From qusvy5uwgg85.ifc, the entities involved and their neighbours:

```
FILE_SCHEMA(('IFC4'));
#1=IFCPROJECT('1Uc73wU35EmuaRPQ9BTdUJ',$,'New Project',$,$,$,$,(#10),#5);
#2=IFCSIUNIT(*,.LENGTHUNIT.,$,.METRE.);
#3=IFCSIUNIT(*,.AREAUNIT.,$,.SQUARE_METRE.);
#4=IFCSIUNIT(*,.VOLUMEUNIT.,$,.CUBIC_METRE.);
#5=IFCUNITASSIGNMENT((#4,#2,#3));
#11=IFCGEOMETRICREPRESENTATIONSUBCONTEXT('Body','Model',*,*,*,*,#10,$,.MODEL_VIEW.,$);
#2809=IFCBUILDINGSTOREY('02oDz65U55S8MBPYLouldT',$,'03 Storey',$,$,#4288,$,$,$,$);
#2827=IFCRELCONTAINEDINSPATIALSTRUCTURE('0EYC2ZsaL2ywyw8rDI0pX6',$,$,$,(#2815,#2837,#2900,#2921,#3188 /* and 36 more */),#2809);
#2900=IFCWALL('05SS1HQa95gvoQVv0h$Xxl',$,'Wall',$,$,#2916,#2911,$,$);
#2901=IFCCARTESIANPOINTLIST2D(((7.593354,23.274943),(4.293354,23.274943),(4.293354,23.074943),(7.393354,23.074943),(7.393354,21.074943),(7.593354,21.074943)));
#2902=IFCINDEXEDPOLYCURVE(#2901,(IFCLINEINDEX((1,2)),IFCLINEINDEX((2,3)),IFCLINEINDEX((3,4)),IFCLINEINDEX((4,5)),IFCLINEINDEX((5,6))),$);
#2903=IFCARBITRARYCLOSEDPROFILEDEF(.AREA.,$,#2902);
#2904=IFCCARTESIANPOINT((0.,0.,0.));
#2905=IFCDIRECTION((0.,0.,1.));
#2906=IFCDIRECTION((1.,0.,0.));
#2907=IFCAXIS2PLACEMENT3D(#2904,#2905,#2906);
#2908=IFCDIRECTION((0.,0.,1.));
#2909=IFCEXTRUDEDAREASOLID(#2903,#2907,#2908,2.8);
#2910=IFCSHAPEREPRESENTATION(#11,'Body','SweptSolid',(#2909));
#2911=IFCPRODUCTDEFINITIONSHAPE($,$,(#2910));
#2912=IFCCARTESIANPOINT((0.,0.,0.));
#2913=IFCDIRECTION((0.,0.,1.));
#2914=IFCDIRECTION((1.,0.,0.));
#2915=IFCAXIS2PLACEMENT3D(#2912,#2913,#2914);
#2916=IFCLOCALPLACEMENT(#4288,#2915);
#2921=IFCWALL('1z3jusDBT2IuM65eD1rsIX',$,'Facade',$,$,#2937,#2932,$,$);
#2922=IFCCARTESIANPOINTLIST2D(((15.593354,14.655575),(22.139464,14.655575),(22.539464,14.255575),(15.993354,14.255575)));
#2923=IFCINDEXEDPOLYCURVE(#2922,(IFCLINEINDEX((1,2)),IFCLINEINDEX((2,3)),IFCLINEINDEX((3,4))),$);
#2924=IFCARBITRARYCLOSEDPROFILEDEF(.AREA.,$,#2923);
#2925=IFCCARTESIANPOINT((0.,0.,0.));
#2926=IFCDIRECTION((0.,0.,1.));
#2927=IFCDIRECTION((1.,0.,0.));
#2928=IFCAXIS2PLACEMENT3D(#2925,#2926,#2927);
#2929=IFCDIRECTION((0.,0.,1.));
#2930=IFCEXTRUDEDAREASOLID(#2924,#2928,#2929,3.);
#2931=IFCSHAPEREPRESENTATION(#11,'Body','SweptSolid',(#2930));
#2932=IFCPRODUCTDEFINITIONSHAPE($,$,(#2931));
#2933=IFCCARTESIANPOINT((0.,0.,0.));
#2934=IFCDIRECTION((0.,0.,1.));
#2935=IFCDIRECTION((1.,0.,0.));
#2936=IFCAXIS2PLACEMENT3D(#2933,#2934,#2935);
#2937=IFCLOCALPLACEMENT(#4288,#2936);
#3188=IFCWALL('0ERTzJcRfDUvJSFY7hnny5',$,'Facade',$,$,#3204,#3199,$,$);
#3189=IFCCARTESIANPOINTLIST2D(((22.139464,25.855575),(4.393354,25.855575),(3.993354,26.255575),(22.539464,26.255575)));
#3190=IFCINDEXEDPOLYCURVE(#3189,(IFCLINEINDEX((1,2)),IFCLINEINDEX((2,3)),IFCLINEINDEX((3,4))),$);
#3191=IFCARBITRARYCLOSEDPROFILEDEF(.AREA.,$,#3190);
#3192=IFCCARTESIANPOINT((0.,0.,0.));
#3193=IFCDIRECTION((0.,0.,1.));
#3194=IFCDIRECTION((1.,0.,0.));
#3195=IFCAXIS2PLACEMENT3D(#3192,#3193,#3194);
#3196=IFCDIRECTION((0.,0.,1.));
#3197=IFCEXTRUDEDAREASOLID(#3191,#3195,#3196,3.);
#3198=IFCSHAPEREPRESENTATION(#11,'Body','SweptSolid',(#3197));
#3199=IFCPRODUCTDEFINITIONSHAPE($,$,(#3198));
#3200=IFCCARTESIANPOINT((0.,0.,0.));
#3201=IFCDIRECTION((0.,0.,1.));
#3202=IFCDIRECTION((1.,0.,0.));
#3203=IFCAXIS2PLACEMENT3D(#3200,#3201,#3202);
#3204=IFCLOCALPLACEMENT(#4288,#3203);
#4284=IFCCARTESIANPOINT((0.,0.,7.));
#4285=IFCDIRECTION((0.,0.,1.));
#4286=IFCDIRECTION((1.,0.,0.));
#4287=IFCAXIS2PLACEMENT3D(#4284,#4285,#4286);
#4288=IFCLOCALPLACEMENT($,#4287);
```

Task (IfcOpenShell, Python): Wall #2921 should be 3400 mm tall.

```python
import ifcopenshell
import ifcopenshell.geom
import ifcopenshell.util.representation
import ifcopenshell.util.shape
import ifcopenshell.util.unit

model = ifcopenshell.open("qusvy5uwgg85.ifc")
unit_scale = ifcopenshell.util.unit.calculate_unit_scale(model)
settings = ifcopenshell.geom.settings()


def volume(element):
    """Net volume in cubic metres, openings subtracted."""
    shape = ifcopenshell.geom.create_shape(settings, element)
    return ifcopenshell.util.shape.get_volume(shape.geometry)


wall = model.by_guid("1z3jusDBT2IuM65eD1rsIX")
before = volume(wall)

body = ifcopenshell.util.representation.get_representation(wall, "Model", "Body")
solid = body.Items[0]
old_height = solid.Depth
solid.Depth = 3.4 / unit_scale
after = volume(wall)

print(f"height {old_height:g} -> {solid.Depth:g}, volume {before:.3f} -> {after:.3f} m3")

model.write("qusvy5uwgg85-out.ifc")
```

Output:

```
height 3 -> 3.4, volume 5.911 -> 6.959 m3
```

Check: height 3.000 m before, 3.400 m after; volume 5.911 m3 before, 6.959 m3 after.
